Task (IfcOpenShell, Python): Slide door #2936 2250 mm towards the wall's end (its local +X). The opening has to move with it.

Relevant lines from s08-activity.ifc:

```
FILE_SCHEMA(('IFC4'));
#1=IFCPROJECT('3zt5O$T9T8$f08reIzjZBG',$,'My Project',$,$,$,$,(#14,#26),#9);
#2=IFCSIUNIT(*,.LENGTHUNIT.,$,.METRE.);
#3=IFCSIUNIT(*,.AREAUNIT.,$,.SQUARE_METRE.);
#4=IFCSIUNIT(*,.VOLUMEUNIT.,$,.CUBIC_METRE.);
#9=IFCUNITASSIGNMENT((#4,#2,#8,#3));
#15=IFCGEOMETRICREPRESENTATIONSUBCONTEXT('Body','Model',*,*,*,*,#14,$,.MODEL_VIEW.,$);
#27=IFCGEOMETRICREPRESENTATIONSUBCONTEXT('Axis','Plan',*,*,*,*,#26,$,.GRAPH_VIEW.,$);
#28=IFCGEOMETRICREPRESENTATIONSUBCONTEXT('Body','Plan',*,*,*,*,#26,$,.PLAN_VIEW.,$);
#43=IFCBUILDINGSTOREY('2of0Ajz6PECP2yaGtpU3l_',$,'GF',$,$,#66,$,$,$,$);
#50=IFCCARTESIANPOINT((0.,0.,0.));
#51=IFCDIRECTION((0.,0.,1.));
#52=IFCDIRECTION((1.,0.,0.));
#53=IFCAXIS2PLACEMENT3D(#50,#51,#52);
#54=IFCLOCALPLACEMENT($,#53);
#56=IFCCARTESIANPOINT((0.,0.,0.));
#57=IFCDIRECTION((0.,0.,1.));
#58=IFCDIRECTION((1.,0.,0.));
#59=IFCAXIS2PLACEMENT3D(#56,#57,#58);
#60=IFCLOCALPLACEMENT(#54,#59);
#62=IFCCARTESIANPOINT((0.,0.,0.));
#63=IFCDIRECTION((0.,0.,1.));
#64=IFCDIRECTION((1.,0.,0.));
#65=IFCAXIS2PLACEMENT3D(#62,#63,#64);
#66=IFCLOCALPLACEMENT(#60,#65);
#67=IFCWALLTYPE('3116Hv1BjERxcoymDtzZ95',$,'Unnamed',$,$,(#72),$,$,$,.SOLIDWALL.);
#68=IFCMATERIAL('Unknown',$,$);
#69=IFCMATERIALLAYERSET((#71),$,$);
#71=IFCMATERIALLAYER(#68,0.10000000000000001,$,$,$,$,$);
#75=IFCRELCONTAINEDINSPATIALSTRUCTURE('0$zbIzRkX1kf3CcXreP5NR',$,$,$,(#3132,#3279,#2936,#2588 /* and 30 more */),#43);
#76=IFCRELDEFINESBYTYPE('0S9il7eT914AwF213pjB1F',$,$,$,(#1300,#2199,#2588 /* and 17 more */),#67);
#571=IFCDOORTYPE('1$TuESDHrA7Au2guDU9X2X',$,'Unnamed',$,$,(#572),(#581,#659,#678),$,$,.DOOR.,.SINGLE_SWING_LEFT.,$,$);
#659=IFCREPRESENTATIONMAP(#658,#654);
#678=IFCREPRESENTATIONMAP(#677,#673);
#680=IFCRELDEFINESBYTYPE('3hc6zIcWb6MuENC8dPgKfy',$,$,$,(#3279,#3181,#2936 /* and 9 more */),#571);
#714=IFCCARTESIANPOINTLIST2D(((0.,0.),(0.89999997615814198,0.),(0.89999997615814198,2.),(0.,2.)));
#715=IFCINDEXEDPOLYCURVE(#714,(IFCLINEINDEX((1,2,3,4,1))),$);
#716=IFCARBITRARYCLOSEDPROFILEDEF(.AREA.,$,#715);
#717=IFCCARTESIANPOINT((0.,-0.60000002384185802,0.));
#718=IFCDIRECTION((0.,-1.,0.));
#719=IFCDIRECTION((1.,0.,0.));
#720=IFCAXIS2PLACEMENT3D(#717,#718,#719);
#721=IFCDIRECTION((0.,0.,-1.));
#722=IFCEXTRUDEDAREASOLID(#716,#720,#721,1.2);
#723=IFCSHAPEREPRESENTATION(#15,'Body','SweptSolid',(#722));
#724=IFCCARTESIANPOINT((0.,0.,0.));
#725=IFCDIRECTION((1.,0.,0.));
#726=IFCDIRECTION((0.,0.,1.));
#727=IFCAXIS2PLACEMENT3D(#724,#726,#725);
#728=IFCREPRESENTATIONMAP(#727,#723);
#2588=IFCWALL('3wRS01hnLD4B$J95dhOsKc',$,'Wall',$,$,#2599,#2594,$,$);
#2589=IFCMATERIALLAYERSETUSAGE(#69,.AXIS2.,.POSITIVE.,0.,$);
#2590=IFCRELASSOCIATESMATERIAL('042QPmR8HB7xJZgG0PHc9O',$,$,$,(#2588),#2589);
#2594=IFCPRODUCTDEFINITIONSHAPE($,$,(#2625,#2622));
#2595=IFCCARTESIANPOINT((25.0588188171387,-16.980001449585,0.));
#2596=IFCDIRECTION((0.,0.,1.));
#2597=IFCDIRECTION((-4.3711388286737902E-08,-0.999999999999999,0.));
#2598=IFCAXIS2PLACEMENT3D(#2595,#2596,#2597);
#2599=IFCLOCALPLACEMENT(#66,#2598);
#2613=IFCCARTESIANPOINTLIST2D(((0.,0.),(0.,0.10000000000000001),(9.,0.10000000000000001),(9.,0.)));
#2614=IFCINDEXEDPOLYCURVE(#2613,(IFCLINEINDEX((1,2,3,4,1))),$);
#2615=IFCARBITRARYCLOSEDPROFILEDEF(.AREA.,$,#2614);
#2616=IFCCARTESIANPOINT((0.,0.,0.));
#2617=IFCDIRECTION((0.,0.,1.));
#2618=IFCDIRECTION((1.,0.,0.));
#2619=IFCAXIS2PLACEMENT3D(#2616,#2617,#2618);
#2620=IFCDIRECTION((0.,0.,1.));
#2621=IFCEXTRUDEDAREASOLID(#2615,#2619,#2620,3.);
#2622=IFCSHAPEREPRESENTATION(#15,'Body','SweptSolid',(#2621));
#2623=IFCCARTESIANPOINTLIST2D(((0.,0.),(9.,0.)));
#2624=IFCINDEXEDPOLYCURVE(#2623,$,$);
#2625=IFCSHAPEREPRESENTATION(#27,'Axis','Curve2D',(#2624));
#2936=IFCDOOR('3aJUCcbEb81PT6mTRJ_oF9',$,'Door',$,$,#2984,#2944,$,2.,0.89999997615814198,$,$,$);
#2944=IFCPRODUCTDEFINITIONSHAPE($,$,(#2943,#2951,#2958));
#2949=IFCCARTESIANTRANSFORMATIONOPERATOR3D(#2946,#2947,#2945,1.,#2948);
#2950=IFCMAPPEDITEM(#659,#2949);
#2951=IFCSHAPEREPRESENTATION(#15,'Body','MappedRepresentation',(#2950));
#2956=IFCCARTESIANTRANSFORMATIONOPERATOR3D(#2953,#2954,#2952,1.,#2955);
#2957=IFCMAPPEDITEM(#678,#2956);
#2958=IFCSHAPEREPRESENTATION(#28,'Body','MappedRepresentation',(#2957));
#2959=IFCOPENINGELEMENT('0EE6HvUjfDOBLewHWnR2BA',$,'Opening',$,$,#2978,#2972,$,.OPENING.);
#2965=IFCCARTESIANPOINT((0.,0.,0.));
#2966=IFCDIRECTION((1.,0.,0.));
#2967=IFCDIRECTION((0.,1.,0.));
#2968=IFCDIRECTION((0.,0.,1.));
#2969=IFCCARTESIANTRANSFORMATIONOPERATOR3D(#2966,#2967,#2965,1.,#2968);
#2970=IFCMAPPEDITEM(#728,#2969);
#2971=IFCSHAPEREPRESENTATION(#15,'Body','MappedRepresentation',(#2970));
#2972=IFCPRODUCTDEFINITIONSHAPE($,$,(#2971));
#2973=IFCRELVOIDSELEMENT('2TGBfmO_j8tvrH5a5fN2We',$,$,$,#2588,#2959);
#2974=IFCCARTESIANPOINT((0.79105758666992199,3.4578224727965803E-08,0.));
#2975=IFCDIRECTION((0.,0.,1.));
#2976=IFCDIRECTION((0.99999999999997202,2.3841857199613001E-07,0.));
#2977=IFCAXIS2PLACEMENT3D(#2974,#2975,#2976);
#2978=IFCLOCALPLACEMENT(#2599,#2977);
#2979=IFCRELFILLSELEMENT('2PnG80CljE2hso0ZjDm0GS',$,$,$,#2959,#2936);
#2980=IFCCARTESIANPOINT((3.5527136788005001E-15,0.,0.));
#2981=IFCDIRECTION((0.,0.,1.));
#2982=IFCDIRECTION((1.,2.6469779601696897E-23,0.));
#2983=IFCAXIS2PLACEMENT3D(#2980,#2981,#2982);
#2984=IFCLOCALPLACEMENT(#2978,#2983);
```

```python
import ifcopenshell
import ifcopenshell.api.geometry
import ifcopenshell.util.placement
import ifcopenshell.util.unit

model = ifcopenshell.open("s08-activity.ifc")
unit_scale = ifcopenshell.util.unit.calculate_unit_scale(model)

door = model.by_guid("3aJUCcbEb81PT6mTRJ_oF9")
opening = door.FillsVoids[0].RelatingOpeningElement
wall = opening.VoidsElements[0].RelatingBuildingElement

wall_matrix = ifcopenshell.util.placement.get_local_placement(wall.ObjectPlacement)
shift = wall_matrix[:3, 0] * 2.25 / unit_scale
before = ifcopenshell.util.placement.get_local_placement(door.ObjectPlacement)[:3, 3].copy()

# The door is placed relative to its opening, so it follows when the opening moves.
matrix = ifcopenshell.util.placement.get_local_placement(opening.ObjectPlacement)
matrix[:3, 3] += shift
ifcopenshell.api.geometry.edit_object_placement(
    model, product=opening, matrix=matrix, is_si=False, should_transform_children=True
)

after = ifcopenshell.util.placement.get_local_placement(door.ObjectPlacement)[:3, 3]
print("door moved by", (after - before).round(3) + 0.0)

model.write("s08-activity_updated.ifc")
```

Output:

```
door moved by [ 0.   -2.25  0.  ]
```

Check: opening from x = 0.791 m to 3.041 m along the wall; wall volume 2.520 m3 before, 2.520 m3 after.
